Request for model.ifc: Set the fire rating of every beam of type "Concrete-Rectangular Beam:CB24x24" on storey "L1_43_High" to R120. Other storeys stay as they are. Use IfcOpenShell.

First a look at what the model holds.

```python
import ifcopenshell
import ifcopenshell.util.element

model = ifcopenshell.open("model.ifc")
print(model.schema)
storey = next(s for s in model.by_type("IfcBuildingStorey") if s.Name == "L1_43_High")
beams = [e for e in ifcopenshell.util.element.get_decomposition(storey) if e.is_a("IfcBeam")]
seen = {}
for e in beams:
    element_type = ifcopenshell.util.element.get_type(e)
    key = (element_type.Name if element_type != e and element_type else None, ifcopenshell.util.element.get_pset(e, "Pset_BeamCommon", "FireRating"))
    seen[key] = seen.get(key, 0) + 1
for (name, value), count in sorted(seen.items(), key=str):
    print(count, "x", name, "|", value)
```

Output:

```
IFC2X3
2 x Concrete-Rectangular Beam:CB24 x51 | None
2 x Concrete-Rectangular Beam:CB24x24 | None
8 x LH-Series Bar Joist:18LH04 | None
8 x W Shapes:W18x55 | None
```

```python
import ifcopenshell
import ifcopenshell.api.pset
import ifcopenshell.util.element

model = ifcopenshell.open("model.ifc")

storey = next(s for s in model.by_type("IfcBuildingStorey") if s.Name == "L1_43_High")
beams = [e for e in ifcopenshell.util.element.get_decomposition(storey) if e.is_a("IfcBeam")]

count = 0
for e in beams:
    element_type = ifcopenshell.util.element.get_type(e)
    if element_type in (None, e) or element_type.Name != "Concrete-Rectangular Beam:CB24x24":
        continue
    # add_pset returns the element's existing set when there is one.
    pset = ifcopenshell.api.pset.add_pset(model, product=e, name="Pset_BeamCommon")
    ifcopenshell.api.pset.edit_pset(model, pset=pset, properties={"FireRating": "R120"})
    count += 1

print(count, "beams updated")

model.write("model-out.ifc")
```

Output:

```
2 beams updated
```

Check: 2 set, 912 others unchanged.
